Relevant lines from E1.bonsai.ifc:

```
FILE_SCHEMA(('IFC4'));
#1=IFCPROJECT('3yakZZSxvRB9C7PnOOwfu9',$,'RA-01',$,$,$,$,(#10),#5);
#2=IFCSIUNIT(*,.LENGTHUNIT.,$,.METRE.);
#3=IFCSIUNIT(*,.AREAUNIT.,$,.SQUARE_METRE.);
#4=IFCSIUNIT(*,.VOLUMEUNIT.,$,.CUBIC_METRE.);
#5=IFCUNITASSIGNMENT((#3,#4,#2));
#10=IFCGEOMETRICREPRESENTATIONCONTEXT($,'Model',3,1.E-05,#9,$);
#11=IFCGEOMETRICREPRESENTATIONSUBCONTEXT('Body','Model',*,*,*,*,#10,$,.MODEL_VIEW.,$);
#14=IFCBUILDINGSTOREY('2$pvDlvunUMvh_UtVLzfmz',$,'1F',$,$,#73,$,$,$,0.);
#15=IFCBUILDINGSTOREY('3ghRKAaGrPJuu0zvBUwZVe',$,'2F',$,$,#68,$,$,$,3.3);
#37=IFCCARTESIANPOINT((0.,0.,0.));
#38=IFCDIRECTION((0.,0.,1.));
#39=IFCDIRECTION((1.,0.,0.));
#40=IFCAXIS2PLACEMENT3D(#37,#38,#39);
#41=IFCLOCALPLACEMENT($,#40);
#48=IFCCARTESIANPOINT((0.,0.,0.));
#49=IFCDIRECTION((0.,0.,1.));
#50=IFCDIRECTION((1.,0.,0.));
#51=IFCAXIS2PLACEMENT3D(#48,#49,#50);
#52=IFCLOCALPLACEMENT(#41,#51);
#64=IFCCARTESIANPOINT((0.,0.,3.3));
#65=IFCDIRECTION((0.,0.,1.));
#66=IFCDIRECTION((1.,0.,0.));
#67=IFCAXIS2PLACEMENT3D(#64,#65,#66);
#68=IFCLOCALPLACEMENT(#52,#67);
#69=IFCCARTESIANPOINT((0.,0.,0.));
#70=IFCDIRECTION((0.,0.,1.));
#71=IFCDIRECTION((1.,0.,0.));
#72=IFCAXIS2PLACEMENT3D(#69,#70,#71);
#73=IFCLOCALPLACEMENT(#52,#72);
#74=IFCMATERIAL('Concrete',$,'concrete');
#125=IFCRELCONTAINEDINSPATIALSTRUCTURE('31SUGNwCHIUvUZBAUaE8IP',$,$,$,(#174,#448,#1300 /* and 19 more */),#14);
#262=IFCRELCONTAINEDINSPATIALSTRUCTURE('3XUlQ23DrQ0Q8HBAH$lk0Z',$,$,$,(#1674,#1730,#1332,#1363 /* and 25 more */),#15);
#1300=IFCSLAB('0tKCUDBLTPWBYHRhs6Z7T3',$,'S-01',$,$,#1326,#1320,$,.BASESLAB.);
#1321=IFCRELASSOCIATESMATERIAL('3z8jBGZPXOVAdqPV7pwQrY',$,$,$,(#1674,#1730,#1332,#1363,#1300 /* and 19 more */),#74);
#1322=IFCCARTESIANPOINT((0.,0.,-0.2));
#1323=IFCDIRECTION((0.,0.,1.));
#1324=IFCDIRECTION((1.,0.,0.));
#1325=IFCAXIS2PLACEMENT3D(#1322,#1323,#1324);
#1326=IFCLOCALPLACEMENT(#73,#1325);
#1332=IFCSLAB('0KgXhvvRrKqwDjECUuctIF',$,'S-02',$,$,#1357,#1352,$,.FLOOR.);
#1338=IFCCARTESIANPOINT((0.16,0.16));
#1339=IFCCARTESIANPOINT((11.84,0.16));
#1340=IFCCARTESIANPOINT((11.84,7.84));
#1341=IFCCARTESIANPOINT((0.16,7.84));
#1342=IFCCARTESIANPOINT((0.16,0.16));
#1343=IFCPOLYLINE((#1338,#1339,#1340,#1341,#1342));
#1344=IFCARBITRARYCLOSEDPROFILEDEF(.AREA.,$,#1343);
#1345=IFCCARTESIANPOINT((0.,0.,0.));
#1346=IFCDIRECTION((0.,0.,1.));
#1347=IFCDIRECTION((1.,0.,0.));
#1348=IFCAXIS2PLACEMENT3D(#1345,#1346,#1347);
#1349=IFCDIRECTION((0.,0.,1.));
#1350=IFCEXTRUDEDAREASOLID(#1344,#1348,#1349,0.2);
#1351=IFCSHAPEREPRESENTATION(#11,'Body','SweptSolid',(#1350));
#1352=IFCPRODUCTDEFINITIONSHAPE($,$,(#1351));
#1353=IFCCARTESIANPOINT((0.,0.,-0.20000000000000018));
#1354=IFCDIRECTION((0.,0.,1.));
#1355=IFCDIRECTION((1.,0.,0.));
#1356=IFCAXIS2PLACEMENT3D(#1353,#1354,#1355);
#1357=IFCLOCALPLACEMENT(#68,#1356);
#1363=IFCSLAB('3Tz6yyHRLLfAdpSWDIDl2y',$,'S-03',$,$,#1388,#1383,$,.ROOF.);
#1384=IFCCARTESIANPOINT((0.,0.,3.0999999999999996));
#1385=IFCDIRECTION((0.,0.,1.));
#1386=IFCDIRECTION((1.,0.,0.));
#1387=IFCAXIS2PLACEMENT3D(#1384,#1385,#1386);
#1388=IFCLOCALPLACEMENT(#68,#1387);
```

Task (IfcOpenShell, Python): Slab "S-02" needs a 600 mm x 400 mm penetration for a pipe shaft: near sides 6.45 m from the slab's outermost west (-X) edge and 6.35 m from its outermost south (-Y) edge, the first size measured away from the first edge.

```python
import numpy as np
import ifcopenshell
import ifcopenshell.api.feature
import ifcopenshell.api.geometry
import ifcopenshell.api.root
import ifcopenshell.geom
import ifcopenshell.util.placement
import ifcopenshell.util.representation
import ifcopenshell.util.shape
import ifcopenshell.util.unit

model = ifcopenshell.open("E1.bonsai.ifc")
unit_scale = ifcopenshell.util.unit.calculate_unit_scale(model)
settings = ifcopenshell.geom.settings()


def volume(element):
    """Net volume in cubic metres, openings subtracted."""
    shape = ifcopenshell.geom.create_shape(settings, element)
    return ifcopenshell.util.shape.get_volume(shape.geometry)


slab = model.by_id(1332)
before = volume(slab)

# Extent in the slab's own axes, in metres. The edges named are its -X and -Y sides.
slab_shape = ifcopenshell.geom.create_shape(settings, slab)
vertices = ifcopenshell.util.shape.get_vertices(slab_shape.geometry)
x_min, y_min, bottom = vertices.min(axis=0)
top = vertices[:, 2].max()

opening = ifcopenshell.api.root.create_entity(model, ifc_class="IfcOpeningElement", name="Pipe shaft opening", predefined_type="OPENING")
context = ifcopenshell.util.representation.get_context(model, "Model", "Body", "MODEL_VIEW")
width, depth = 0.6, 0.4
outline = [(0.0, 0.0), (width, 0.0), (width, depth), (0.0, depth), (0.0, 0.0)]
# Overshoot both faces by 50 mm so the cut is clean.
shape = ifcopenshell.api.geometry.add_slab_representation(
    model, context=context, depth=top - bottom + 0.1, polyline=outline
)
ifcopenshell.api.geometry.assign_representation(model, product=opening, representation=shape)

matrix = ifcopenshell.util.placement.get_local_placement(slab.ObjectPlacement)
matrix[:, 3] = matrix @ np.append(np.array([x_min + 6.45, y_min + 6.35, bottom - 0.05]) / unit_scale, 1.0)
ifcopenshell.api.geometry.edit_object_placement(model, product=opening, matrix=matrix, is_si=False)
ifcopenshell.api.feature.add_feature(model, feature=opening, element=slab)

after = volume(slab)

print(f"slab volume {before:.3f} -> {after:.3f} m3")

model.write("E1.bonsai_rev.ifc")
```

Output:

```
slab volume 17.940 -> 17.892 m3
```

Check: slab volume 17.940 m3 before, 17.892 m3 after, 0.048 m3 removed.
